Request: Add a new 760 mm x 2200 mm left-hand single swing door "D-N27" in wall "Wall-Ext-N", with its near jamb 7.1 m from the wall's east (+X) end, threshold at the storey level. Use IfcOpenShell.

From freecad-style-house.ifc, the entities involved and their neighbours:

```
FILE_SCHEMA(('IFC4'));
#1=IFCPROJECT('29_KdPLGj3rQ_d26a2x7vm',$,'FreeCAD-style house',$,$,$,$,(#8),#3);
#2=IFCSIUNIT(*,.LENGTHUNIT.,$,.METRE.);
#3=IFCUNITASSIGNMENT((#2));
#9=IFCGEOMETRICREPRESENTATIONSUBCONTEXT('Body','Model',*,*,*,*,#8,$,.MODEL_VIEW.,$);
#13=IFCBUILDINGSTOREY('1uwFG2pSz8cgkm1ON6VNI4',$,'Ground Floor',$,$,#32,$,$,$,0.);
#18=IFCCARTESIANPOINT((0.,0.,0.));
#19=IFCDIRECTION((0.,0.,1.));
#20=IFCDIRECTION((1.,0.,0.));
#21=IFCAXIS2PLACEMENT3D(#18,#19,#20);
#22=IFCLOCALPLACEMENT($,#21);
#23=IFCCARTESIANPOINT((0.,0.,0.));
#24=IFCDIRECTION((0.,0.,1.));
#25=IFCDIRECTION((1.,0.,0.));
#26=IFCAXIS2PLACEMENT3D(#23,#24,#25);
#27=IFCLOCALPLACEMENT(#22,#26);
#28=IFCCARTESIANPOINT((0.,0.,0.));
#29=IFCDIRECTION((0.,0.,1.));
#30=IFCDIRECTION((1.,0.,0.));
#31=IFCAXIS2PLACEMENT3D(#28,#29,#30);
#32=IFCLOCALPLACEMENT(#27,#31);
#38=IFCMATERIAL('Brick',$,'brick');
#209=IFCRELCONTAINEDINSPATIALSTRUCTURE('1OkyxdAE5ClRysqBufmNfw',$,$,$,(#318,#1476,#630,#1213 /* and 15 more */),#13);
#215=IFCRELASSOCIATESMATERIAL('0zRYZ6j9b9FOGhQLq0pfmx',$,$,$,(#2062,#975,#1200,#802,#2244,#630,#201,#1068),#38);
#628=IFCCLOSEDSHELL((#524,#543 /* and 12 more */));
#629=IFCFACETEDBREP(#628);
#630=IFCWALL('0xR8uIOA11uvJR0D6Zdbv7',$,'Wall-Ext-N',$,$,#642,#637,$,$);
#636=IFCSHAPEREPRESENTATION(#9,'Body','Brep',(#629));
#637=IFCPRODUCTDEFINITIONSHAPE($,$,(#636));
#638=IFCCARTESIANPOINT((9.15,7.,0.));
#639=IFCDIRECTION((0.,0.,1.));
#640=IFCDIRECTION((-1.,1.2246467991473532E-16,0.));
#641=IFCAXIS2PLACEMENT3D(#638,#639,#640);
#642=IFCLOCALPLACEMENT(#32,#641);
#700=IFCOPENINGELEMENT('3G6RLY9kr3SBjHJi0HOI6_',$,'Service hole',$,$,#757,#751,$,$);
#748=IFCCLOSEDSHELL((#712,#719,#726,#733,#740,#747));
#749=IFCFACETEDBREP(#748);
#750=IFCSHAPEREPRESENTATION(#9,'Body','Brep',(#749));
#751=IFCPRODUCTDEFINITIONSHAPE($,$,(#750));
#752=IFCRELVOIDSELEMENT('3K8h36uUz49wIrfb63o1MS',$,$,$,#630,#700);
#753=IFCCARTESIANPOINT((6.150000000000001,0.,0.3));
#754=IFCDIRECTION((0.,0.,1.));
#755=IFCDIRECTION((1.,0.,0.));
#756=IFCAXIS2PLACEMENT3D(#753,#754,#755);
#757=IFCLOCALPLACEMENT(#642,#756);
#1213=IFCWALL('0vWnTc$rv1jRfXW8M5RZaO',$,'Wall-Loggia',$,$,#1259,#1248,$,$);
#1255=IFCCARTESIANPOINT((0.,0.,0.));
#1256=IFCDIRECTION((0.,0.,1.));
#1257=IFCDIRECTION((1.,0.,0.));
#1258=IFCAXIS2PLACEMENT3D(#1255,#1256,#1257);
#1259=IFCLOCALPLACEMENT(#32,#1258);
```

```python
import numpy as np
import ifcopenshell
import ifcopenshell.api.feature
import ifcopenshell.api.geometry
import ifcopenshell.api.root
import ifcopenshell.api.spatial
import ifcopenshell.geom
import ifcopenshell.util.element
import ifcopenshell.util.placement
import ifcopenshell.util.representation
import ifcopenshell.util.shape
import ifcopenshell.util.unit

model = ifcopenshell.open("freecad-style-house.ifc")
unit_scale = ifcopenshell.util.unit.calculate_unit_scale(model)
settings = ifcopenshell.geom.settings()


def volume(element):
    """Net volume in cubic metres, openings subtracted."""
    shape = ifcopenshell.geom.create_shape(settings, element)
    return ifcopenshell.util.shape.get_volume(shape.geometry)


wall = model.by_id(630)
storey = ifcopenshell.util.element.get_container(wall, ifc_class="IfcBuildingStorey")
context = ifcopenshell.util.representation.get_context(model, "Model", "Body", "MODEL_VIEW")
before = volume(wall)

width, height, from_end, sill = 0.76, 2.2, 7.1, 0.0  # metres

# The wall runs along its own X axis, and the end named is its -X end.
wall_shape = ifcopenshell.geom.create_shape(settings, wall)
x, y, z = ifcopenshell.util.shape.get_vertices(wall_shape.geometry).T
start = x.min() + from_end
face, thickness = float(y.min()), float(y.max() - y.min())
wall_matrix = ifcopenshell.util.placement.get_local_placement(wall.ObjectPlacement)
level = ifcopenshell.util.placement.get_local_placement(storey.ObjectPlacement)[2, 3]


def in_wall(x, y):
    """Placement at x, y metres in the wall's axes, at sill height."""
    matrix = wall_matrix.copy()
    matrix[:, 3] = wall_matrix @ np.array([x / unit_scale, y / unit_scale, 0.0, 1.0])
    matrix[2, 3] = level + sill / unit_scale
    return matrix


# Opening: a box that overshoots both wall faces by 50 mm.
opening = ifcopenshell.api.root.create_entity(model, ifc_class="IfcOpeningElement", predefined_type="OPENING")
box = ifcopenshell.api.geometry.add_wall_representation(
    model, context=context, length=width, height=height, thickness=thickness + 0.1
)
ifcopenshell.api.geometry.assign_representation(model, product=opening, representation=box)
ifcopenshell.api.geometry.edit_object_placement(model, product=opening, matrix=in_wall(start, face - 0.05), is_si=False)
ifcopenshell.api.feature.add_feature(model, feature=opening, element=wall)

door = ifcopenshell.api.root.create_entity(model, ifc_class="IfcDoor", name="D-N27", predefined_type="DOOR")
door.OverallWidth, door.OverallHeight = width / unit_scale, height / unit_scale
door.OperationType = "SINGLE_SWING_LEFT"
body = ifcopenshell.api.geometry.add_door_representation(
    model,
    context=context,
    overall_width=door.OverallWidth,
    overall_height=door.OverallHeight,
    operation_type="SINGLE_SWING_LEFT",
    lining_properties={"LiningDepth": thickness / unit_scale, "ThresholdDepth": thickness / unit_scale},
)
ifcopenshell.api.geometry.assign_representation(model, product=door, representation=body)
ifcopenshell.api.spatial.assign_container(model, products=[door], relating_structure=storey)
ifcopenshell.api.feature.add_filling(model, opening=opening, element=door)

# The lining spans the wall, so the door starts at the wall face.
ifcopenshell.api.geometry.edit_object_placement(model, product=door, matrix=in_wall(start, face), is_si=False)

after = volume(wall)

print(f"wall volume {before:.3f} -> {after:.3f} m3")

model.write("freecad-style-house_rev.ifc")
```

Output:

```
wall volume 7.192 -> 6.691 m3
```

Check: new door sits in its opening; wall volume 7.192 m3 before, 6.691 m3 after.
